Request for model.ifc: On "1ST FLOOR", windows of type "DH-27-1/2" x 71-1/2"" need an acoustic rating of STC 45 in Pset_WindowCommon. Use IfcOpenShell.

First a look at what the model holds.

```python
import ifcopenshell
import ifcopenshell.util.element

model = ifcopenshell.open("model.ifc")
print(model.schema)
storey = next(s for s in model.by_type("IfcBuildingStorey") if s.Name == "1ST FLOOR")
windows = [e for e in ifcopenshell.util.element.get_decomposition(storey) if e.is_a("IfcWindow")]
seen = {}
for e in windows:
    element_type = ifcopenshell.util.element.get_type(e)
    key = (element_type.Name if element_type != e and element_type else None, ifcopenshell.util.element.get_pset(e, "Pset_WindowCommon", "AcousticRating"))
    seen[key] = seen.get(key, 0) + 1
for (name, value), count in sorted(seen.items(), key=str):
    print(count, "x", name, "|", value)
```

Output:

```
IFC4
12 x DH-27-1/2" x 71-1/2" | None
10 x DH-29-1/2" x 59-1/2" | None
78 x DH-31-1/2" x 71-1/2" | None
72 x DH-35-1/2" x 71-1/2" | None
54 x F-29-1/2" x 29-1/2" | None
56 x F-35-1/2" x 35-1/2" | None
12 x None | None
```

```python
import ifcopenshell
import ifcopenshell.api.pset
import ifcopenshell.util.element

model = ifcopenshell.open("model.ifc")

storey = next(s for s in model.by_type("IfcBuildingStorey") if s.Name == "1ST FLOOR")
windows = [e for e in ifcopenshell.util.element.get_decomposition(storey) if e.is_a("IfcWindow")]

count = 0
for e in windows:
    element_type = ifcopenshell.util.element.get_type(e)
    if element_type in (None, e) or element_type.Name != 'DH-27-1/2" x 71-1/2"':
        continue
    # add_pset returns the element's existing set when there is one.
    pset = ifcopenshell.api.pset.add_pset(model, product=e, name="Pset_WindowCommon")
    ifcopenshell.api.pset.edit_pset(model, pset=pset, properties={"AcousticRating": "STC 45"})
    count += 1

print(count, "windows updated")

model.write("model_rev.ifc")
```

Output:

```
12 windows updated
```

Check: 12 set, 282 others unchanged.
